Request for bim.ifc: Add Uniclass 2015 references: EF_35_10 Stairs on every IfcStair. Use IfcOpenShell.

First a look at what the model holds.

```python
import ifcopenshell

model = ifcopenshell.open("bim.ifc")
print(model.schema)
print("classifications:", [c.Name for c in model.by_type("IfcClassification")])
for ifc_class in ("IfcDoor", "IfcRoof", "IfcStair", "IfcWall", "IfcWindow"):
    print(ifc_class, len(model.by_type(ifc_class)))
```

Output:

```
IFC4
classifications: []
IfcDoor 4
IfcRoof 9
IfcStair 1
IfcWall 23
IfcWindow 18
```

```python
import ifcopenshell
import ifcopenshell.api.classification

model = ifcopenshell.open("bim.ifc")

system = ifcopenshell.api.classification.add_classification(model, classification="Uniclass 2015")

codes = {
    "IfcStair": ("EF_35_10", "Stairs"),
}
for ifc_class, (code, name) in codes.items():
    products = model.by_type(ifc_class)
    ifcopenshell.api.classification.add_reference(
        model, products=products, classification=system, identification=code, name=name
    )
    print(code, len(products))

model.write("bim_v2.ifc")
```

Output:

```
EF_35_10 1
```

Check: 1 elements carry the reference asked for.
